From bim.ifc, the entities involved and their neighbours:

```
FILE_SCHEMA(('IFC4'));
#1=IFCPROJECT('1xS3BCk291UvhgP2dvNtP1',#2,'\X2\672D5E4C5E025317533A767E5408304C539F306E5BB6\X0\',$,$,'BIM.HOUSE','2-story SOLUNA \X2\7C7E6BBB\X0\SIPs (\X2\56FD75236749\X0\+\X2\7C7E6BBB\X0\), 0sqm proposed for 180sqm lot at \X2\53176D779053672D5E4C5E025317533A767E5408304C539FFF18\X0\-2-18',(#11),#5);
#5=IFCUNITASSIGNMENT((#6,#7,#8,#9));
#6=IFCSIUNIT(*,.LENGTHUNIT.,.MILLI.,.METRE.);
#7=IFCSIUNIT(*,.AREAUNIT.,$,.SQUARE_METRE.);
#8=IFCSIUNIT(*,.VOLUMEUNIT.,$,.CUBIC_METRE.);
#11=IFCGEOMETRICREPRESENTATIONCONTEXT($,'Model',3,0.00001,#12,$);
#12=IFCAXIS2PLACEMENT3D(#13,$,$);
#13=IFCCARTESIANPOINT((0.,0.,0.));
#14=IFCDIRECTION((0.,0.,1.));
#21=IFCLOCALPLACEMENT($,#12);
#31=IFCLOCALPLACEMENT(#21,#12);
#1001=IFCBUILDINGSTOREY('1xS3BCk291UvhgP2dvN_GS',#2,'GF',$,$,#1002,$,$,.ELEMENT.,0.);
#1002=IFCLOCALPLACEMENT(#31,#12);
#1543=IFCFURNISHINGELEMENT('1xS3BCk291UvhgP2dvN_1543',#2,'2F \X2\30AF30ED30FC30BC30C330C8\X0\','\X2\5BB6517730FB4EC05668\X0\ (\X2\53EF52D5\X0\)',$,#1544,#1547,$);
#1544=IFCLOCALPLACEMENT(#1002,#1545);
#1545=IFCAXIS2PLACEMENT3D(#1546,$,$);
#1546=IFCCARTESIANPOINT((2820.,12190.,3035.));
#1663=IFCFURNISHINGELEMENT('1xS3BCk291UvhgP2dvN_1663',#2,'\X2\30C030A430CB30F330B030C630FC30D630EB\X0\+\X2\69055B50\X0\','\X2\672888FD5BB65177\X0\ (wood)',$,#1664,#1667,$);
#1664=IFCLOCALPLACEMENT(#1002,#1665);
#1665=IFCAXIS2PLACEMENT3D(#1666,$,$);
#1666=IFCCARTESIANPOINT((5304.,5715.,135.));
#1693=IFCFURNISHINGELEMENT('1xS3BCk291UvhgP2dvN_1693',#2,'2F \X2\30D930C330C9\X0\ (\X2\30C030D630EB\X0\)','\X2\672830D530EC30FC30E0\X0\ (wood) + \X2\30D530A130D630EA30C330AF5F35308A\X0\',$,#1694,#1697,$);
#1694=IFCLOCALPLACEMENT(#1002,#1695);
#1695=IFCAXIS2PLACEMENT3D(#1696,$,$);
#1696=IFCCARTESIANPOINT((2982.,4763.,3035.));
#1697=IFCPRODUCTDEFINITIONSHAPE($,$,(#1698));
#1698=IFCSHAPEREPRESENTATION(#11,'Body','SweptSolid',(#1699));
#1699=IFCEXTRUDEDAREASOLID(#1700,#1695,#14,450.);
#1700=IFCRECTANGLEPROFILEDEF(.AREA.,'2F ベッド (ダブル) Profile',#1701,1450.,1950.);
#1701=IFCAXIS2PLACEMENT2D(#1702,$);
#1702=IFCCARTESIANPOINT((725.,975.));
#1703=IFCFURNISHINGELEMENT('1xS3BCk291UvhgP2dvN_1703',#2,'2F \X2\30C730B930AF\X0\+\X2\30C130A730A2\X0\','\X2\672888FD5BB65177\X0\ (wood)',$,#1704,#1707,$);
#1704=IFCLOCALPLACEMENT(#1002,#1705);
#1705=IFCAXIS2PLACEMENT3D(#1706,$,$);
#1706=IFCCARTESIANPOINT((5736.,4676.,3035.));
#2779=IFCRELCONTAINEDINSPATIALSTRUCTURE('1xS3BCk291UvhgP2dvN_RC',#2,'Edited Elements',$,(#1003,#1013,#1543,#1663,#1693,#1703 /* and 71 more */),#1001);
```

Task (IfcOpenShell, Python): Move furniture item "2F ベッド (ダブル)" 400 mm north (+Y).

```python
import ifcopenshell
import ifcopenshell.api.geometry
import ifcopenshell.util.placement
import ifcopenshell.util.unit

model = ifcopenshell.open("bim.ifc")
unit_scale = ifcopenshell.util.unit.calculate_unit_scale(model)

item = model.by_guid("1xS3BCk291UvhgP2dvN_1693")
matrix = ifcopenshell.util.placement.get_local_placement(item.ObjectPlacement)
matrix[1, 3] += 0.4 / unit_scale
ifcopenshell.api.geometry.edit_object_placement(model, product=item, matrix=matrix, is_si=False)

print(ifcopenshell.util.placement.get_local_placement(item.ObjectPlacement).round(3) + 0.0)

model.write("bim_rev.ifc")
```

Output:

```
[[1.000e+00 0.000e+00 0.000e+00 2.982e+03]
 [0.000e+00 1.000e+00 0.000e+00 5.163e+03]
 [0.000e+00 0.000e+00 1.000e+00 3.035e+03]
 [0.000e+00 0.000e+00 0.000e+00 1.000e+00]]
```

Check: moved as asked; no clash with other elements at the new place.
